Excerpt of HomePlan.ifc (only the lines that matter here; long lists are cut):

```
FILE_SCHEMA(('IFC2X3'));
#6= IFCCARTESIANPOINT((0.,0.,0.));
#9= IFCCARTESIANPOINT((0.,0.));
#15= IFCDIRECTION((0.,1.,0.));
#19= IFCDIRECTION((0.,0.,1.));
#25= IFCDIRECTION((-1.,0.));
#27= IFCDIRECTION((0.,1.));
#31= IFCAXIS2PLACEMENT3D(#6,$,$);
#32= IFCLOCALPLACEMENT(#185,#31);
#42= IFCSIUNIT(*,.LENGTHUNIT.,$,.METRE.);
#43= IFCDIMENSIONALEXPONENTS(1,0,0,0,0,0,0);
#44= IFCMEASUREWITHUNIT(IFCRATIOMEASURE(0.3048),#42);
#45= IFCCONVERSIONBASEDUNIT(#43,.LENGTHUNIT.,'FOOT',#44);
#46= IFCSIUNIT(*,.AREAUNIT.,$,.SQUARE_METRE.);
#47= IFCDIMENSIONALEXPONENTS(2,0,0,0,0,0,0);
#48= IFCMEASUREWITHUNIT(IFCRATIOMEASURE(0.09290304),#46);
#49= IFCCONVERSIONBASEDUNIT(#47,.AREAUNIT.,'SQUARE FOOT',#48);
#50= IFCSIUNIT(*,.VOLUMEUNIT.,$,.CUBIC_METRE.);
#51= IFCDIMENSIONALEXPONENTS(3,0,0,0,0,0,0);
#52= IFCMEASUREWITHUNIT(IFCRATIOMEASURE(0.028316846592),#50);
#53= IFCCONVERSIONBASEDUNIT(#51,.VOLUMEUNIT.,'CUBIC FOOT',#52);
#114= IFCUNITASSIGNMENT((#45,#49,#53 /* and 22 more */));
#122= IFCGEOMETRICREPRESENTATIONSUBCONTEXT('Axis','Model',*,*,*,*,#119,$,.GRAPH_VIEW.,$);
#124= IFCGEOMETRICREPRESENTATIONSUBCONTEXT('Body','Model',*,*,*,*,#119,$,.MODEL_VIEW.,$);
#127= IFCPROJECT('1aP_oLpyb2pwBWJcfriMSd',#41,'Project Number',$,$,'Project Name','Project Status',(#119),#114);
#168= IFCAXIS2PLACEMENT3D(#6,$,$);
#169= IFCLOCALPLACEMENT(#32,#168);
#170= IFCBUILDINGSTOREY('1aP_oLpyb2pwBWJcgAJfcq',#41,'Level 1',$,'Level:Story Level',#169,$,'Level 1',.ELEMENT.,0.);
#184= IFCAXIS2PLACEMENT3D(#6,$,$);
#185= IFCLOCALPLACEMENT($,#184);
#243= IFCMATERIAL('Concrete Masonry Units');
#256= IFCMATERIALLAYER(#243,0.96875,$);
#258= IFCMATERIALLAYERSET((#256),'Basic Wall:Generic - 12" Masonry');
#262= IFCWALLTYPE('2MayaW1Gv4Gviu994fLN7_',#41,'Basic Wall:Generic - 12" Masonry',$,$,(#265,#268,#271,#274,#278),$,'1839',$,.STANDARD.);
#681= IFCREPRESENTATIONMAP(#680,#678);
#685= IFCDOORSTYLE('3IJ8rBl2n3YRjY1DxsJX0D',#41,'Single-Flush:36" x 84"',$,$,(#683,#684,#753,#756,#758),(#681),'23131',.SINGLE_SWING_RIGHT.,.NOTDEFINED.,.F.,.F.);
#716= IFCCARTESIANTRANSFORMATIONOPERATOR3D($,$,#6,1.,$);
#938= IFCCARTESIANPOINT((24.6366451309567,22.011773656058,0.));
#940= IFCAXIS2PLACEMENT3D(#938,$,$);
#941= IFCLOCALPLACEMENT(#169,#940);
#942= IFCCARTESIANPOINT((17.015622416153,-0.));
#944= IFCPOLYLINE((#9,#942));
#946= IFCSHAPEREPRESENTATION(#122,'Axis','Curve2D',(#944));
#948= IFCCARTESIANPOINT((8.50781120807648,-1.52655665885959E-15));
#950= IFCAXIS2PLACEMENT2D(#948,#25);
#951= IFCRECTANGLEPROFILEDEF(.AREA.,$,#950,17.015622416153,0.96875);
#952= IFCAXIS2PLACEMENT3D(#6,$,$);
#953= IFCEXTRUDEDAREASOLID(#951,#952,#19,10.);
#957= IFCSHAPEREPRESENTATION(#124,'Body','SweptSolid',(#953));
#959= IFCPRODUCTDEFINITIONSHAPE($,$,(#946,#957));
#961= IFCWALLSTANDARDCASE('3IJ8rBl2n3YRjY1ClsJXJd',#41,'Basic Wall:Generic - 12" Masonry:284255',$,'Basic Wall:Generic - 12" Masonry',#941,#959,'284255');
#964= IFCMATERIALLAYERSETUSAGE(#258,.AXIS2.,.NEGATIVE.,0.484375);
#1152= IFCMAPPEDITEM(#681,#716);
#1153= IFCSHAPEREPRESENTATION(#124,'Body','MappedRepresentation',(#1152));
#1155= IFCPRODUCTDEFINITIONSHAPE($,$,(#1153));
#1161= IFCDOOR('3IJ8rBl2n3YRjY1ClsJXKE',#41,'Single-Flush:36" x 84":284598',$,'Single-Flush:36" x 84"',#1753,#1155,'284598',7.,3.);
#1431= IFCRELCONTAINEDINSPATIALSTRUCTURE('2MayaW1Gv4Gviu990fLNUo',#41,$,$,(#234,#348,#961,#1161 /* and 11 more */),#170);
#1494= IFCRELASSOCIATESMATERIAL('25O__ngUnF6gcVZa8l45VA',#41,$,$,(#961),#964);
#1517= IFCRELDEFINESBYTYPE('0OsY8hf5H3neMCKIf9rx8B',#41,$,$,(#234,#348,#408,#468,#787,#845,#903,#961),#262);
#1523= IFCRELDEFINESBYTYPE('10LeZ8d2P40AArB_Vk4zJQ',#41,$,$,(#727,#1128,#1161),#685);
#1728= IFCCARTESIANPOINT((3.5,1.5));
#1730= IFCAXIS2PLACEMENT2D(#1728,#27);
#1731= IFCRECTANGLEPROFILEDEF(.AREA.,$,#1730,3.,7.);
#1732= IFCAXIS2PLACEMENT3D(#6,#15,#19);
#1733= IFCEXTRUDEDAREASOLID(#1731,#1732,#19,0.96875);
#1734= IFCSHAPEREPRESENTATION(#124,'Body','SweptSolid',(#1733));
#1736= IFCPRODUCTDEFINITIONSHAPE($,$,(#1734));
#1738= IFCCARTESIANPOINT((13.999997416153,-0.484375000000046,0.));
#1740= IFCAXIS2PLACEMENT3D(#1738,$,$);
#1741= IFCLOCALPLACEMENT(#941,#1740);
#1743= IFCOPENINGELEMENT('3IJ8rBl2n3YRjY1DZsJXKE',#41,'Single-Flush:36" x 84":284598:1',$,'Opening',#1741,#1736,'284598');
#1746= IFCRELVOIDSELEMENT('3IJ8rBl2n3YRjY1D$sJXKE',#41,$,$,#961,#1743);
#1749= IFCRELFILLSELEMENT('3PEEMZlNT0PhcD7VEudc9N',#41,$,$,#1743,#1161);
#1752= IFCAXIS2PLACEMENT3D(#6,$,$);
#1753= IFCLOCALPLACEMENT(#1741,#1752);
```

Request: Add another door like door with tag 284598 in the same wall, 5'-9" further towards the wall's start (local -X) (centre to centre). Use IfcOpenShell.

```python
import ifcopenshell
import ifcopenshell.api.feature
import ifcopenshell.api.geometry
import ifcopenshell.api.root
import ifcopenshell.geom
import ifcopenshell.util.element
import ifcopenshell.util.placement
import ifcopenshell.util.shape
import ifcopenshell.util.unit

model = ifcopenshell.open("HomePlan.ifc")
unit_scale = ifcopenshell.util.unit.calculate_unit_scale(model)
settings = ifcopenshell.geom.settings()


def volume(element):
    """Net volume in cubic metres, openings subtracted."""
    shape = ifcopenshell.geom.create_shape(settings, element)
    return ifcopenshell.util.shape.get_volume(shape.geometry)


def reuse_history(source, copy):
    """copy_class also copies each property set's owner history, people and application; keep the originals."""
    for rel in copy.IsDefinedBy:
        if rel.is_a("IfcRelDefinesByProperties") and (history := rel.RelatingPropertyDefinition.OwnerHistory):
            rel.RelatingPropertyDefinition.OwnerHistory = source.OwnerHistory
            ifcopenshell.util.element.remove_deep2(model, history)


door = model.by_id(1161)
opening = door.FillsVoids[0].RelatingOpeningElement
wall = opening.VoidsElements[0].RelatingBuildingElement
before = volume(wall)
shift = ifcopenshell.util.placement.get_local_placement(wall.ObjectPlacement)[:3, 0] * -69 * 0.0254 / unit_scale

# copy_class copies the void relationship, type, container and properties, but no geometry.
new_opening = ifcopenshell.api.root.copy_class(model, product=opening)
new_opening.Representation = ifcopenshell.util.element.copy_deep(
    model, opening.Representation, exclude=["IfcGeometricRepresentationContext", "IfcRepresentationMap"]
)
new_opening.Name = 'Single-Flush:36" x 84"'
new_opening.Tag = None
new_door = ifcopenshell.api.root.copy_class(model, product=door)
new_door.Representation = ifcopenshell.util.element.copy_deep(
    model, door.Representation, exclude=["IfcGeometricRepresentationContext", "IfcRepresentationMap"]
)
new_door.Name = 'Single-Flush:36" x 84"'
new_door.Tag = None
reuse_history(door, new_door)
fills = ifcopenshell.api.feature.add_filling(model, opening=new_opening, element=new_door)
fills.OwnerHistory = new_door.OwnerHistory  # required in IFC2X3

for old, new in ((opening, new_opening), (door, new_door)):
    matrix = ifcopenshell.util.placement.get_local_placement(old.ObjectPlacement)
    matrix[:3, 3] += shift
    ifcopenshell.api.geometry.edit_object_placement(model, product=new, matrix=matrix, is_si=False)

after = volume(wall)

print(f"wall volume {before:.3f} -> {after:.3f} m3")

model.write("HomePlan_updated.ifc")
```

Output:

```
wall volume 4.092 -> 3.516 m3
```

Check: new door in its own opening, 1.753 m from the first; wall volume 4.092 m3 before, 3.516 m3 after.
